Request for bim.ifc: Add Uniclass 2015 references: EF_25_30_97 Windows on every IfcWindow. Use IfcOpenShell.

First a look at what the model holds.

```python
import ifcopenshell

model = ifcopenshell.open("bim.ifc")
print(model.schema)
print("classifications:", [c.Name for c in model.by_type("IfcClassification")])
for ifc_class in ("IfcDoor", "IfcRoof", "IfcStair", "IfcWall", "IfcWindow"):
    print(ifc_class, len(model.by_type(ifc_class)))
```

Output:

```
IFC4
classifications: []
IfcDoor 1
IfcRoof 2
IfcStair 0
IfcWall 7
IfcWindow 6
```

```python
import ifcopenshell
import ifcopenshell.api.classification

model = ifcopenshell.open("bim.ifc")

system = ifcopenshell.api.classification.add_classification(model, classification="Uniclass 2015")

codes = {
    "IfcWindow": ("EF_25_30_97", "Windows"),
}
for ifc_class, (code, name) in codes.items():
    products = model.by_type(ifc_class)
    ifcopenshell.api.classification.add_reference(
        model, products=products, classification=system, identification=code, name=name
    )
    print(code, len(products))

model.write("bim_rev.ifc")
```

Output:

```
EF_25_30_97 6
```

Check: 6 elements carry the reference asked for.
